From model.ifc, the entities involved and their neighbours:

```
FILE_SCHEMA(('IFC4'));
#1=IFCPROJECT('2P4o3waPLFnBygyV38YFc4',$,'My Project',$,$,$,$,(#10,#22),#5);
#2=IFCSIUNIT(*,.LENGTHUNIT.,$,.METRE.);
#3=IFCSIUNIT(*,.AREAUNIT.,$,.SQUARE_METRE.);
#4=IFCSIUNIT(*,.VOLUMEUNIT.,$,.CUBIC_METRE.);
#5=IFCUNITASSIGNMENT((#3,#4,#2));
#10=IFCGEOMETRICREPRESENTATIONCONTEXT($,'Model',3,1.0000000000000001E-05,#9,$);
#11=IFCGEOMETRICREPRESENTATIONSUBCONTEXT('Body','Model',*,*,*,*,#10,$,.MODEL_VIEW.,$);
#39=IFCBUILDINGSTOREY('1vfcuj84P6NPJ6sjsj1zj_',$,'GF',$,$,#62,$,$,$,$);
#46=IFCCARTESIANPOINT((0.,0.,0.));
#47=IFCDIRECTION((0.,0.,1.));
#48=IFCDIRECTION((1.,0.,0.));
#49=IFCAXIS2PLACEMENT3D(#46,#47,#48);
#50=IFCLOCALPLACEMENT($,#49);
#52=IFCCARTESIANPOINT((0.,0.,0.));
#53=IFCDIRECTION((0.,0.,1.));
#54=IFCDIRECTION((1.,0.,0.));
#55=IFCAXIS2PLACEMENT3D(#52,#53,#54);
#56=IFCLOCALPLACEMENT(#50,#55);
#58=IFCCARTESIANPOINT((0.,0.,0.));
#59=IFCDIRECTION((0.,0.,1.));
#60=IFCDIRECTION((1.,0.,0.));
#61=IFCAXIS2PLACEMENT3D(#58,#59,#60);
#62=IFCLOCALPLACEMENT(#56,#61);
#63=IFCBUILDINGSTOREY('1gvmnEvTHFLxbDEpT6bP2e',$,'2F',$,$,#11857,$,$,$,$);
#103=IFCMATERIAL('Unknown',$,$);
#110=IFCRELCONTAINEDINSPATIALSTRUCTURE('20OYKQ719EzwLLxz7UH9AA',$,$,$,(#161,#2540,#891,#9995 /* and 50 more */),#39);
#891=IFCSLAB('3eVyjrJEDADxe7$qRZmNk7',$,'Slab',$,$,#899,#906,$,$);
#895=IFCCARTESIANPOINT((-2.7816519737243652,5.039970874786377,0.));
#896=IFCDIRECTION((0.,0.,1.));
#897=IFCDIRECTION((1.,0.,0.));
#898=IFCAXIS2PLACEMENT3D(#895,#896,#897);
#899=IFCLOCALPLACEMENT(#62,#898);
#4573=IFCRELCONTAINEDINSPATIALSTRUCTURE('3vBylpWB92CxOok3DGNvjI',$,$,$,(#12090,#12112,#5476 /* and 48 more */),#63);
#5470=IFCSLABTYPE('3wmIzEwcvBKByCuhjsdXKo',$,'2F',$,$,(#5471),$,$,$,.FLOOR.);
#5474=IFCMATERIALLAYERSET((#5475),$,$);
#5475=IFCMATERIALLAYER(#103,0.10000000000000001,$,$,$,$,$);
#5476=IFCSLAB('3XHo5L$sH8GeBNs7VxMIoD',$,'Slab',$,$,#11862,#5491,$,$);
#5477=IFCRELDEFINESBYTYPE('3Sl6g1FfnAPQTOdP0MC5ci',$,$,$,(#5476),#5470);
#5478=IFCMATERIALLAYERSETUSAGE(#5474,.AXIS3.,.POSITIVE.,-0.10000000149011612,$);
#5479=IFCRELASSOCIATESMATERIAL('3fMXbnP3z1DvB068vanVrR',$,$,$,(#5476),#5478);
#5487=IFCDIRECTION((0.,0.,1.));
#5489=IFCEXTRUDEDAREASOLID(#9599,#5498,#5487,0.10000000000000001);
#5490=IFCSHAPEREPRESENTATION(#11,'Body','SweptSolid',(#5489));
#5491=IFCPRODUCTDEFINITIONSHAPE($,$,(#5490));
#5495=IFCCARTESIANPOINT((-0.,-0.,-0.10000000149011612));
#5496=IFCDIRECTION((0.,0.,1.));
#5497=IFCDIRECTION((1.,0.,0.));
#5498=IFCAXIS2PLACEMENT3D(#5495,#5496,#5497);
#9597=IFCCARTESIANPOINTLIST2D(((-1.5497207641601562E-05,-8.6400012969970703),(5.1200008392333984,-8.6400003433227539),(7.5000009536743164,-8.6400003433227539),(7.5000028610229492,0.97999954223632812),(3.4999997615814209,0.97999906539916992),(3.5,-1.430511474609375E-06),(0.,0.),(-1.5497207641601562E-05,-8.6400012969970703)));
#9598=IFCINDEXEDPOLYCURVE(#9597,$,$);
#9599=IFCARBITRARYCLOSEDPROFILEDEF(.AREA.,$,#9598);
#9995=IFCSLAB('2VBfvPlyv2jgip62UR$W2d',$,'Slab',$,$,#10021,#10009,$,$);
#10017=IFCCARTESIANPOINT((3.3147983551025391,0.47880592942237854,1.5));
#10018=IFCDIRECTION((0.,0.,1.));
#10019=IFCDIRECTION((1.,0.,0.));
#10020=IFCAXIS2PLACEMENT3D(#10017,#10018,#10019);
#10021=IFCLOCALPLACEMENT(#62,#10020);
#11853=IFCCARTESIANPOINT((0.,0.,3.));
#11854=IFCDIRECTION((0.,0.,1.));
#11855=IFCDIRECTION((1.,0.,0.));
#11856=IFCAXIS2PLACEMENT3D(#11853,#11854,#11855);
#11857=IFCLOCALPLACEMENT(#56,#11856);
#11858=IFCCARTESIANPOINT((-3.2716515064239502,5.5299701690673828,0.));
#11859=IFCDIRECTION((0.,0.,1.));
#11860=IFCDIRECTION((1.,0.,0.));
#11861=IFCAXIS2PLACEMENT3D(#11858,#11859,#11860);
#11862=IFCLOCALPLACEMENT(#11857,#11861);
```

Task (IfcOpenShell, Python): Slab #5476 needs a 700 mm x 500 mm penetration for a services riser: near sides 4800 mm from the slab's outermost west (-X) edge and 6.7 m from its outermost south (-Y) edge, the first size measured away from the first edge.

```python
import numpy as np
import ifcopenshell
import ifcopenshell.api.feature
import ifcopenshell.api.geometry
import ifcopenshell.api.root
import ifcopenshell.geom
import ifcopenshell.util.placement
import ifcopenshell.util.representation
import ifcopenshell.util.shape
import ifcopenshell.util.unit

model = ifcopenshell.open("model.ifc")
unit_scale = ifcopenshell.util.unit.calculate_unit_scale(model)
settings = ifcopenshell.geom.settings()


def volume(element):
    """Net volume in cubic metres, openings subtracted."""
    shape = ifcopenshell.geom.create_shape(settings, element)
    return ifcopenshell.util.shape.get_volume(shape.geometry)


slab = model.by_guid("3XHo5L$sH8GeBNs7VxMIoD")
before = volume(slab)

# Extent in the slab's own axes, in metres. The edges named are its -X and -Y sides.
slab_shape = ifcopenshell.geom.create_shape(settings, slab)
vertices = ifcopenshell.util.shape.get_vertices(slab_shape.geometry)
x_min, y_min, bottom = vertices.min(axis=0)
top = vertices[:, 2].max()

opening = ifcopenshell.api.root.create_entity(model, ifc_class="IfcOpeningElement", name="Services riser opening", predefined_type="OPENING")
context = ifcopenshell.util.representation.get_context(model, "Model", "Body", "MODEL_VIEW")
width, depth = 0.7, 0.5
outline = [(0.0, 0.0), (width, 0.0), (width, depth), (0.0, depth), (0.0, 0.0)]
# Overshoot both faces by 50 mm so the cut is clean.
shape = ifcopenshell.api.geometry.add_slab_representation(
    model, context=context, depth=top - bottom + 0.1, polyline=outline
)
ifcopenshell.api.geometry.assign_representation(model, product=opening, representation=shape)

matrix = ifcopenshell.util.placement.get_local_placement(slab.ObjectPlacement)
matrix[:, 3] = matrix @ np.append(np.array([x_min + 4.8, y_min + 6.7, bottom - 0.05]) / unit_scale, 1.0)
ifcopenshell.api.geometry.edit_object_placement(model, product=opening, matrix=matrix, is_si=False)
ifcopenshell.api.feature.add_feature(model, feature=opening, element=slab)

after = volume(slab)

print(f"slab volume {before:.3f} -> {after:.3f} m3")

model.write("model_v2.ifc")
```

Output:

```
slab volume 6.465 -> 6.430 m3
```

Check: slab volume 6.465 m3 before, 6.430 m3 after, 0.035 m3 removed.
